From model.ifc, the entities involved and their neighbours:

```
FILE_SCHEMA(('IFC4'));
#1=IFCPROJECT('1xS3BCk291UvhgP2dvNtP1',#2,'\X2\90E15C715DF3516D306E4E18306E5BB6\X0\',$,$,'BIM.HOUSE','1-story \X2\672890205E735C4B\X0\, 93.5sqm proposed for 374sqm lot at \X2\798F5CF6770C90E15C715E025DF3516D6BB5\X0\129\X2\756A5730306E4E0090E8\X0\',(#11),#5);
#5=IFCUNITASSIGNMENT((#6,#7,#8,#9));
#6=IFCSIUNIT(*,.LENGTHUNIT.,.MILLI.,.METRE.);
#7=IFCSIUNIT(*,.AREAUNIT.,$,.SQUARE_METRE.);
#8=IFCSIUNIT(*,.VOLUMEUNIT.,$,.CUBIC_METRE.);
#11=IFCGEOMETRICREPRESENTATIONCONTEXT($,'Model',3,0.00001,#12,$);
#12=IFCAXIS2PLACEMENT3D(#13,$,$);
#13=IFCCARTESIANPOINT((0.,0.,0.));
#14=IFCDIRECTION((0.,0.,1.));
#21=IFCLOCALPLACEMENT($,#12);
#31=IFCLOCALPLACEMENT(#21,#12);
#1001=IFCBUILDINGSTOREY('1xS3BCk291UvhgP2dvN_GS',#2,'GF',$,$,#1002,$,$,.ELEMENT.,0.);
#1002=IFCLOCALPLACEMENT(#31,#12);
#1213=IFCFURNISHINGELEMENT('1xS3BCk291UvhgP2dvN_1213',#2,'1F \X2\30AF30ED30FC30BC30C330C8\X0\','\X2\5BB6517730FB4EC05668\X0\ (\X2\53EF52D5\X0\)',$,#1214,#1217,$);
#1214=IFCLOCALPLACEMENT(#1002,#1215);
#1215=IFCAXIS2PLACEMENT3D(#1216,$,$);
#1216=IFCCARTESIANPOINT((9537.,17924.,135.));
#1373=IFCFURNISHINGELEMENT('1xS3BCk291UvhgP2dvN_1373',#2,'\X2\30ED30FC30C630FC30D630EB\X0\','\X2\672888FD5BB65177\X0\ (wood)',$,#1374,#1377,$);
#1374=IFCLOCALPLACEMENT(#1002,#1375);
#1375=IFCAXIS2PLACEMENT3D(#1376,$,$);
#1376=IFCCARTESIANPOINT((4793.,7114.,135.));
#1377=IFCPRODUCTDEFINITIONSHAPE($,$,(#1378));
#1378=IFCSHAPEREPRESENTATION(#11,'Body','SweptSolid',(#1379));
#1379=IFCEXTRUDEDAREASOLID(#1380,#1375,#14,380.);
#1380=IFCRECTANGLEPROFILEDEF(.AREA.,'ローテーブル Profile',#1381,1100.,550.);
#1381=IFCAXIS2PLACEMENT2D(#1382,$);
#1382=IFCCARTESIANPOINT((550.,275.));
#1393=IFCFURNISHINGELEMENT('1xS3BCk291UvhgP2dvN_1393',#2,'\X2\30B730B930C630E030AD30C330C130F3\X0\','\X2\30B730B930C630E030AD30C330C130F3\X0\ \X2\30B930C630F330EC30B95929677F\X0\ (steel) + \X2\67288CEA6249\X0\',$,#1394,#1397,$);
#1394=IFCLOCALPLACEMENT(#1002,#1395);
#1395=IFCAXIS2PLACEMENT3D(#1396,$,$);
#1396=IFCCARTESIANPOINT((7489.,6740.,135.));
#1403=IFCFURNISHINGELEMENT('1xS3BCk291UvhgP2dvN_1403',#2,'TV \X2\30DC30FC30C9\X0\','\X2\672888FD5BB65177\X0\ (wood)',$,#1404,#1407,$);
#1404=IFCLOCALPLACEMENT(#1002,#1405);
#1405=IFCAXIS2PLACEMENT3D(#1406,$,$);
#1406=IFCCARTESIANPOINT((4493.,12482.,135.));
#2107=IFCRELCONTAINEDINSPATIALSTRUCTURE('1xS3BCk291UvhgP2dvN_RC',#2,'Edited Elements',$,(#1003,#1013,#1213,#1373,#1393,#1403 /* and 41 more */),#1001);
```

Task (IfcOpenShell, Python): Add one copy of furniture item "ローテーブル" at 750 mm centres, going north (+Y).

```python
import numpy as np
import ifcopenshell
import ifcopenshell.api.geometry
import ifcopenshell.api.root
import ifcopenshell.util.element
import ifcopenshell.util.placement
import ifcopenshell.util.unit

model = ifcopenshell.open("model.ifc")
unit_scale = ifcopenshell.util.unit.calculate_unit_scale(model)


def reuse_history(source, copy):
    """copy_class also copies each property set's owner history, people and application; keep the originals."""
    for rel in copy.IsDefinedBy:
        if rel.is_a("IfcRelDefinesByProperties") and (history := rel.RelatingPropertyDefinition.OwnerHistory):
            rel.RelatingPropertyDefinition.OwnerHistory = source.OwnerHistory
            ifcopenshell.util.element.remove_deep2(model, history)


source = model.by_guid("1xS3BCk291UvhgP2dvN_1373")
base = ifcopenshell.util.placement.get_local_placement(source.ObjectPlacement)
step = np.array([0.0, 1.0, 0.0]) * 0.75 / unit_scale

for i in range(1, 2):
    copy = ifcopenshell.api.root.copy_class(model, product=source)
    copy.Representation = ifcopenshell.util.element.copy_deep(
        model, source.Representation, exclude=["IfcGeometricRepresentationContext", "IfcRepresentationMap"]
    )
    reuse_history(source, copy)
    matrix = base.copy()
    matrix[:3, 3] += i * step
    print("added at", matrix[:3, 3].round(3) + 0.0)
    ifcopenshell.api.geometry.edit_object_placement(model, product=copy, matrix=matrix, is_si=False)

model.write("model_rev.ifc")
```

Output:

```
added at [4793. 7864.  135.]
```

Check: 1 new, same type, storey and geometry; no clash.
